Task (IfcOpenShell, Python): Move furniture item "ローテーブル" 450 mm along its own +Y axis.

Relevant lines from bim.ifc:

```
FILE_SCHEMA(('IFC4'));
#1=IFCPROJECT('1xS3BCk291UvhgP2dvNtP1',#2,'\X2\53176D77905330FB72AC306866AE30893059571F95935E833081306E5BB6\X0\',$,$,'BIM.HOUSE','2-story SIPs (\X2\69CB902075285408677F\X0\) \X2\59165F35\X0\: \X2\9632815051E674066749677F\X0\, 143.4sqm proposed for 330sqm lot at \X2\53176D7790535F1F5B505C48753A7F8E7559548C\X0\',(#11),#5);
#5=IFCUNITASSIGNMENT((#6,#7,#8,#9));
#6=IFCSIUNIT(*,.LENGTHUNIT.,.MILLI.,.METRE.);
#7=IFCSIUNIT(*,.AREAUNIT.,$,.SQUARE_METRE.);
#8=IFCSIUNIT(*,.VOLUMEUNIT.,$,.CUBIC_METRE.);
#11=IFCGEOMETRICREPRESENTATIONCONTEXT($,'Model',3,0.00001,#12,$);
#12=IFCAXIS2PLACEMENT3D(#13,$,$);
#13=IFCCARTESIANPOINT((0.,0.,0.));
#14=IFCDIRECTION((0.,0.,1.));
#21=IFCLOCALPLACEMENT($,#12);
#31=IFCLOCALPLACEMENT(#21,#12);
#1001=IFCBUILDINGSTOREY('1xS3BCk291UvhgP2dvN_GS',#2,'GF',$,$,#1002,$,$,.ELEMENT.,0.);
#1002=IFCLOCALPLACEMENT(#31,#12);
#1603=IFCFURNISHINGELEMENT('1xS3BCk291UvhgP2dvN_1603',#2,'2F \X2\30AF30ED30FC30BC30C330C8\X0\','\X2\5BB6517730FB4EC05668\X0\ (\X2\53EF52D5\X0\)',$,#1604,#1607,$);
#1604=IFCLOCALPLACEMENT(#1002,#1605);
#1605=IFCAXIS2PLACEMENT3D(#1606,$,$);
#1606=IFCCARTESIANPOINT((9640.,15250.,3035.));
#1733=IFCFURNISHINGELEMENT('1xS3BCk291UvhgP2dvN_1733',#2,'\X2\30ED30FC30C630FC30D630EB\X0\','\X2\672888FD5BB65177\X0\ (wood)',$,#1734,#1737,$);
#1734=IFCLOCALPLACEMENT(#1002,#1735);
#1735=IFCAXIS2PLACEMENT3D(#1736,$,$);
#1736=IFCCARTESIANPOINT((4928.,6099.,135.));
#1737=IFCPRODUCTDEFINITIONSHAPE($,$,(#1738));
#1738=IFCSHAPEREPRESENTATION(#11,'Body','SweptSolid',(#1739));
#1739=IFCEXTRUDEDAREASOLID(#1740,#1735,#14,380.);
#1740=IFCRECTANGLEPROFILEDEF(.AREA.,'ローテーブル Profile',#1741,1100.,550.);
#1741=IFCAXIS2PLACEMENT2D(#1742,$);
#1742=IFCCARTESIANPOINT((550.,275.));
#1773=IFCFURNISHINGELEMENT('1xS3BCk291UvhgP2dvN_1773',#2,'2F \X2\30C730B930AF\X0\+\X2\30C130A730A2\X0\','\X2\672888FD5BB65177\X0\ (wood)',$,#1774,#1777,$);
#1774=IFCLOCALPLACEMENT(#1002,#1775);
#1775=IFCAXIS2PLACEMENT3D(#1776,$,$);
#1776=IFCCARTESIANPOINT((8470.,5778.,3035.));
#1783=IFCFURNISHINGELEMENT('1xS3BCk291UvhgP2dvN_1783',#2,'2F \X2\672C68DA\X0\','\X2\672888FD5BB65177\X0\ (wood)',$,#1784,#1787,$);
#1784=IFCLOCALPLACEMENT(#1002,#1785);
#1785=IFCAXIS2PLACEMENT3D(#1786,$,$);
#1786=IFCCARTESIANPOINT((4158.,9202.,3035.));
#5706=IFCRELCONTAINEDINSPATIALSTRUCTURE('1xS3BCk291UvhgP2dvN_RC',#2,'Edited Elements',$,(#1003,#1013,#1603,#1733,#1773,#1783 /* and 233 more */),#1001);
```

```python
import ifcopenshell
import ifcopenshell.api.geometry
import ifcopenshell.util.placement

model = ifcopenshell.open("bim.ifc")

item = model.by_id(1733)
matrix = ifcopenshell.util.placement.get_local_placement(item.ObjectPlacement)
matrix[:3, 3] += matrix[:3, 1] * 450.0
ifcopenshell.api.geometry.edit_object_placement(model, product=item, matrix=matrix, is_si=False)

print(ifcopenshell.util.placement.get_local_placement(item.ObjectPlacement).round(3) + 0.0)

model.write("bim_rev.ifc")
```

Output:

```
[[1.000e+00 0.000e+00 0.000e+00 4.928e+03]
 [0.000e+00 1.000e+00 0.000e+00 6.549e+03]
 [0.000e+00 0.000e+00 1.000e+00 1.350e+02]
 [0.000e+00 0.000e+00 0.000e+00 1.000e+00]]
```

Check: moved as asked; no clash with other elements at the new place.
